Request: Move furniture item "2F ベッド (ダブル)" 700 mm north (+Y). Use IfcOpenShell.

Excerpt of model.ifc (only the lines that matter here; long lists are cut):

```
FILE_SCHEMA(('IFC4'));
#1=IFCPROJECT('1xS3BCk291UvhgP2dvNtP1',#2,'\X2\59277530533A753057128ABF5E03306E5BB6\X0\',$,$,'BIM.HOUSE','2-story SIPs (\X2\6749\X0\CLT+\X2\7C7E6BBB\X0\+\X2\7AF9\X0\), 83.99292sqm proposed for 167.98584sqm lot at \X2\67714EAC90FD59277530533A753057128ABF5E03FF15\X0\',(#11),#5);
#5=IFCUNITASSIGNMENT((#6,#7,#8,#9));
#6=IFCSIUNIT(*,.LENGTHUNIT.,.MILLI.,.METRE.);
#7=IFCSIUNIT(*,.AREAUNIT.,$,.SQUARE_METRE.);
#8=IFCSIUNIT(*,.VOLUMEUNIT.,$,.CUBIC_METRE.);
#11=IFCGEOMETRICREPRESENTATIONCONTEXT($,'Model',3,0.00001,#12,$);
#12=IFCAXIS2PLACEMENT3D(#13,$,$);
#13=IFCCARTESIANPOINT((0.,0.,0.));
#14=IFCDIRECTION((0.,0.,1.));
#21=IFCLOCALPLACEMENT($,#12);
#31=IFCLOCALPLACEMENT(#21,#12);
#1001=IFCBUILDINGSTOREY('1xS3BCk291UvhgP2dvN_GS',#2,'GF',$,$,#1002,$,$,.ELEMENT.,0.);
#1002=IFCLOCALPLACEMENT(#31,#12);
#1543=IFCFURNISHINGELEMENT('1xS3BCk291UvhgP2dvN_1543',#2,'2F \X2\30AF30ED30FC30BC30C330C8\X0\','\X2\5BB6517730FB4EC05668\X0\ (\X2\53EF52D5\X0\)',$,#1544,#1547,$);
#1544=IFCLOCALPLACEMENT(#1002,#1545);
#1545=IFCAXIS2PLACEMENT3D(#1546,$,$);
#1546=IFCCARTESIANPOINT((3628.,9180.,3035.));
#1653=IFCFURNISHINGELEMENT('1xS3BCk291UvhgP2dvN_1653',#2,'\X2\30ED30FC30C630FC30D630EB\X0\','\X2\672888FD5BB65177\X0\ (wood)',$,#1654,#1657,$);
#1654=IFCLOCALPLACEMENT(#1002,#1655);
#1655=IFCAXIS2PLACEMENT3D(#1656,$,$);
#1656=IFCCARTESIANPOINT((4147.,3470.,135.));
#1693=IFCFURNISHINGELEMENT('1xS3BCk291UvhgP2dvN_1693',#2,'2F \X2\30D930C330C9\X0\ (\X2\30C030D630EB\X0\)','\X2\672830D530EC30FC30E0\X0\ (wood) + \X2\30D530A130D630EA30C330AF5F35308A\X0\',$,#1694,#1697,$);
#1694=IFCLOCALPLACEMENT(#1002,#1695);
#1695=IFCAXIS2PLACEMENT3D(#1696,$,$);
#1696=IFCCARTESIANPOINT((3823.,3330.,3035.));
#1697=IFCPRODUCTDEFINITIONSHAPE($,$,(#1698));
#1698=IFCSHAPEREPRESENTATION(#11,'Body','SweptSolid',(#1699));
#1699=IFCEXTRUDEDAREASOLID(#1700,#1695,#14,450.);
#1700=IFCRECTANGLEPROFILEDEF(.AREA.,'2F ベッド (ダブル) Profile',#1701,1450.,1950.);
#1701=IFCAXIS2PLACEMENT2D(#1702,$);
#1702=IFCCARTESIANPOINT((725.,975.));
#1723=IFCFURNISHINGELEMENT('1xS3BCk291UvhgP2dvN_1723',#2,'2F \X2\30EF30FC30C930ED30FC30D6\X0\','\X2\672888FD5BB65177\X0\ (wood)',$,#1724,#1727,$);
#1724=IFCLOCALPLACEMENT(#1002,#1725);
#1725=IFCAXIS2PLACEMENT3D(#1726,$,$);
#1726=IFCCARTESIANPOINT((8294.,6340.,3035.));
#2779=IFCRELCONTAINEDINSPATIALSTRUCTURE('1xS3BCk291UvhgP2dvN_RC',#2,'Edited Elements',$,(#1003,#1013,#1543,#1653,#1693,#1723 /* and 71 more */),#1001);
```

```python
import ifcopenshell
import ifcopenshell.api.geometry
import ifcopenshell.util.placement

model = ifcopenshell.open("model.ifc")

item = model.by_guid("1xS3BCk291UvhgP2dvN_1693")
matrix = ifcopenshell.util.placement.get_local_placement(item.ObjectPlacement)
matrix[1, 3] += 700.0
ifcopenshell.api.geometry.edit_object_placement(model, product=item, matrix=matrix, is_si=False)

print(ifcopenshell.util.placement.get_local_placement(item.ObjectPlacement).round(3) + 0.0)

model.write("model_rev.ifc")
```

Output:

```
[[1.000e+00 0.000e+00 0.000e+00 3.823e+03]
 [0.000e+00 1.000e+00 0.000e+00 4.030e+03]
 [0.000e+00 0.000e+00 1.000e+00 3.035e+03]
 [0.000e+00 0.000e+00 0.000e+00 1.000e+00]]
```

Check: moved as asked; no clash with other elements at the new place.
